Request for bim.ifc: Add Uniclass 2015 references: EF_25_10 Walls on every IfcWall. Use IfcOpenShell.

First a look at what the model holds.

```python
import ifcopenshell

model = ifcopenshell.open("bim.ifc")
print(model.schema)
print("classifications:", [c.Name for c in model.by_type("IfcClassification")])
for ifc_class in ("IfcDoor", "IfcRoof", "IfcStair", "IfcWall", "IfcWindow"):
    print(ifc_class, len(model.by_type(ifc_class)))
```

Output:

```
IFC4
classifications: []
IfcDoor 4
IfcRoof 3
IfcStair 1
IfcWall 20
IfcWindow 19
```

```python
import ifcopenshell
import ifcopenshell.api.classification

model = ifcopenshell.open("bim.ifc")

system = ifcopenshell.api.classification.add_classification(model, classification="Uniclass 2015")

codes = {
    "IfcWall": ("EF_25_10", "Walls"),
}
for ifc_class, (code, name) in codes.items():
    products = model.by_type(ifc_class)
    ifcopenshell.api.classification.add_reference(
        model, products=products, classification=system, identification=code, name=name
    )
    print(code, len(products))

model.write("bim-out.ifc")
```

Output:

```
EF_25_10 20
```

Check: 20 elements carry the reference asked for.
